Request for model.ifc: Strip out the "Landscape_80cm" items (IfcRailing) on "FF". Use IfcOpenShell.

First a look at what the model holds.

```python
import ifcopenshell
import ifcopenshell.util.element

model = ifcopenshell.open("model.ifc")
print(model.schema)
storey = next(s for s in model.by_type("IfcBuildingStorey") if s.Name == "FF")
railings = [e for e in ifcopenshell.util.element.get_decomposition(storey) if e.is_a("IfcRailing")]
seen = {}
for e in railings:
    element_type = ifcopenshell.util.element.get_type(e)
    name = element_type.Name if element_type not in (None, e) else None
    seen[name] = seen.get(name, 0) + 1
for name, count in sorted(seen.items(), key=str):
    print(count, "x", name)
```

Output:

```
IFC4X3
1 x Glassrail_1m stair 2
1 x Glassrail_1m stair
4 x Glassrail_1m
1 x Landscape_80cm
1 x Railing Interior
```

```python
import ifcopenshell
import ifcopenshell.api.root
import ifcopenshell.util.element

model = ifcopenshell.open("model.ifc")

storey = next(s for s in model.by_type("IfcBuildingStorey") if s.Name == "FF")
railings = [e for e in ifcopenshell.util.element.get_decomposition(storey) if e.is_a("IfcRailing")]
targets = [e for e in railings if (t := ifcopenshell.util.element.get_type(e)) not in (None, e) and t.Name == "Landscape_80cm"]

for e in targets:
    ifcopenshell.api.root.remove_product(model, product=e)
print(len(targets), "removed")

model.write("model_updated.ifc")
```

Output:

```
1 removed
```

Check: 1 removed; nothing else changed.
